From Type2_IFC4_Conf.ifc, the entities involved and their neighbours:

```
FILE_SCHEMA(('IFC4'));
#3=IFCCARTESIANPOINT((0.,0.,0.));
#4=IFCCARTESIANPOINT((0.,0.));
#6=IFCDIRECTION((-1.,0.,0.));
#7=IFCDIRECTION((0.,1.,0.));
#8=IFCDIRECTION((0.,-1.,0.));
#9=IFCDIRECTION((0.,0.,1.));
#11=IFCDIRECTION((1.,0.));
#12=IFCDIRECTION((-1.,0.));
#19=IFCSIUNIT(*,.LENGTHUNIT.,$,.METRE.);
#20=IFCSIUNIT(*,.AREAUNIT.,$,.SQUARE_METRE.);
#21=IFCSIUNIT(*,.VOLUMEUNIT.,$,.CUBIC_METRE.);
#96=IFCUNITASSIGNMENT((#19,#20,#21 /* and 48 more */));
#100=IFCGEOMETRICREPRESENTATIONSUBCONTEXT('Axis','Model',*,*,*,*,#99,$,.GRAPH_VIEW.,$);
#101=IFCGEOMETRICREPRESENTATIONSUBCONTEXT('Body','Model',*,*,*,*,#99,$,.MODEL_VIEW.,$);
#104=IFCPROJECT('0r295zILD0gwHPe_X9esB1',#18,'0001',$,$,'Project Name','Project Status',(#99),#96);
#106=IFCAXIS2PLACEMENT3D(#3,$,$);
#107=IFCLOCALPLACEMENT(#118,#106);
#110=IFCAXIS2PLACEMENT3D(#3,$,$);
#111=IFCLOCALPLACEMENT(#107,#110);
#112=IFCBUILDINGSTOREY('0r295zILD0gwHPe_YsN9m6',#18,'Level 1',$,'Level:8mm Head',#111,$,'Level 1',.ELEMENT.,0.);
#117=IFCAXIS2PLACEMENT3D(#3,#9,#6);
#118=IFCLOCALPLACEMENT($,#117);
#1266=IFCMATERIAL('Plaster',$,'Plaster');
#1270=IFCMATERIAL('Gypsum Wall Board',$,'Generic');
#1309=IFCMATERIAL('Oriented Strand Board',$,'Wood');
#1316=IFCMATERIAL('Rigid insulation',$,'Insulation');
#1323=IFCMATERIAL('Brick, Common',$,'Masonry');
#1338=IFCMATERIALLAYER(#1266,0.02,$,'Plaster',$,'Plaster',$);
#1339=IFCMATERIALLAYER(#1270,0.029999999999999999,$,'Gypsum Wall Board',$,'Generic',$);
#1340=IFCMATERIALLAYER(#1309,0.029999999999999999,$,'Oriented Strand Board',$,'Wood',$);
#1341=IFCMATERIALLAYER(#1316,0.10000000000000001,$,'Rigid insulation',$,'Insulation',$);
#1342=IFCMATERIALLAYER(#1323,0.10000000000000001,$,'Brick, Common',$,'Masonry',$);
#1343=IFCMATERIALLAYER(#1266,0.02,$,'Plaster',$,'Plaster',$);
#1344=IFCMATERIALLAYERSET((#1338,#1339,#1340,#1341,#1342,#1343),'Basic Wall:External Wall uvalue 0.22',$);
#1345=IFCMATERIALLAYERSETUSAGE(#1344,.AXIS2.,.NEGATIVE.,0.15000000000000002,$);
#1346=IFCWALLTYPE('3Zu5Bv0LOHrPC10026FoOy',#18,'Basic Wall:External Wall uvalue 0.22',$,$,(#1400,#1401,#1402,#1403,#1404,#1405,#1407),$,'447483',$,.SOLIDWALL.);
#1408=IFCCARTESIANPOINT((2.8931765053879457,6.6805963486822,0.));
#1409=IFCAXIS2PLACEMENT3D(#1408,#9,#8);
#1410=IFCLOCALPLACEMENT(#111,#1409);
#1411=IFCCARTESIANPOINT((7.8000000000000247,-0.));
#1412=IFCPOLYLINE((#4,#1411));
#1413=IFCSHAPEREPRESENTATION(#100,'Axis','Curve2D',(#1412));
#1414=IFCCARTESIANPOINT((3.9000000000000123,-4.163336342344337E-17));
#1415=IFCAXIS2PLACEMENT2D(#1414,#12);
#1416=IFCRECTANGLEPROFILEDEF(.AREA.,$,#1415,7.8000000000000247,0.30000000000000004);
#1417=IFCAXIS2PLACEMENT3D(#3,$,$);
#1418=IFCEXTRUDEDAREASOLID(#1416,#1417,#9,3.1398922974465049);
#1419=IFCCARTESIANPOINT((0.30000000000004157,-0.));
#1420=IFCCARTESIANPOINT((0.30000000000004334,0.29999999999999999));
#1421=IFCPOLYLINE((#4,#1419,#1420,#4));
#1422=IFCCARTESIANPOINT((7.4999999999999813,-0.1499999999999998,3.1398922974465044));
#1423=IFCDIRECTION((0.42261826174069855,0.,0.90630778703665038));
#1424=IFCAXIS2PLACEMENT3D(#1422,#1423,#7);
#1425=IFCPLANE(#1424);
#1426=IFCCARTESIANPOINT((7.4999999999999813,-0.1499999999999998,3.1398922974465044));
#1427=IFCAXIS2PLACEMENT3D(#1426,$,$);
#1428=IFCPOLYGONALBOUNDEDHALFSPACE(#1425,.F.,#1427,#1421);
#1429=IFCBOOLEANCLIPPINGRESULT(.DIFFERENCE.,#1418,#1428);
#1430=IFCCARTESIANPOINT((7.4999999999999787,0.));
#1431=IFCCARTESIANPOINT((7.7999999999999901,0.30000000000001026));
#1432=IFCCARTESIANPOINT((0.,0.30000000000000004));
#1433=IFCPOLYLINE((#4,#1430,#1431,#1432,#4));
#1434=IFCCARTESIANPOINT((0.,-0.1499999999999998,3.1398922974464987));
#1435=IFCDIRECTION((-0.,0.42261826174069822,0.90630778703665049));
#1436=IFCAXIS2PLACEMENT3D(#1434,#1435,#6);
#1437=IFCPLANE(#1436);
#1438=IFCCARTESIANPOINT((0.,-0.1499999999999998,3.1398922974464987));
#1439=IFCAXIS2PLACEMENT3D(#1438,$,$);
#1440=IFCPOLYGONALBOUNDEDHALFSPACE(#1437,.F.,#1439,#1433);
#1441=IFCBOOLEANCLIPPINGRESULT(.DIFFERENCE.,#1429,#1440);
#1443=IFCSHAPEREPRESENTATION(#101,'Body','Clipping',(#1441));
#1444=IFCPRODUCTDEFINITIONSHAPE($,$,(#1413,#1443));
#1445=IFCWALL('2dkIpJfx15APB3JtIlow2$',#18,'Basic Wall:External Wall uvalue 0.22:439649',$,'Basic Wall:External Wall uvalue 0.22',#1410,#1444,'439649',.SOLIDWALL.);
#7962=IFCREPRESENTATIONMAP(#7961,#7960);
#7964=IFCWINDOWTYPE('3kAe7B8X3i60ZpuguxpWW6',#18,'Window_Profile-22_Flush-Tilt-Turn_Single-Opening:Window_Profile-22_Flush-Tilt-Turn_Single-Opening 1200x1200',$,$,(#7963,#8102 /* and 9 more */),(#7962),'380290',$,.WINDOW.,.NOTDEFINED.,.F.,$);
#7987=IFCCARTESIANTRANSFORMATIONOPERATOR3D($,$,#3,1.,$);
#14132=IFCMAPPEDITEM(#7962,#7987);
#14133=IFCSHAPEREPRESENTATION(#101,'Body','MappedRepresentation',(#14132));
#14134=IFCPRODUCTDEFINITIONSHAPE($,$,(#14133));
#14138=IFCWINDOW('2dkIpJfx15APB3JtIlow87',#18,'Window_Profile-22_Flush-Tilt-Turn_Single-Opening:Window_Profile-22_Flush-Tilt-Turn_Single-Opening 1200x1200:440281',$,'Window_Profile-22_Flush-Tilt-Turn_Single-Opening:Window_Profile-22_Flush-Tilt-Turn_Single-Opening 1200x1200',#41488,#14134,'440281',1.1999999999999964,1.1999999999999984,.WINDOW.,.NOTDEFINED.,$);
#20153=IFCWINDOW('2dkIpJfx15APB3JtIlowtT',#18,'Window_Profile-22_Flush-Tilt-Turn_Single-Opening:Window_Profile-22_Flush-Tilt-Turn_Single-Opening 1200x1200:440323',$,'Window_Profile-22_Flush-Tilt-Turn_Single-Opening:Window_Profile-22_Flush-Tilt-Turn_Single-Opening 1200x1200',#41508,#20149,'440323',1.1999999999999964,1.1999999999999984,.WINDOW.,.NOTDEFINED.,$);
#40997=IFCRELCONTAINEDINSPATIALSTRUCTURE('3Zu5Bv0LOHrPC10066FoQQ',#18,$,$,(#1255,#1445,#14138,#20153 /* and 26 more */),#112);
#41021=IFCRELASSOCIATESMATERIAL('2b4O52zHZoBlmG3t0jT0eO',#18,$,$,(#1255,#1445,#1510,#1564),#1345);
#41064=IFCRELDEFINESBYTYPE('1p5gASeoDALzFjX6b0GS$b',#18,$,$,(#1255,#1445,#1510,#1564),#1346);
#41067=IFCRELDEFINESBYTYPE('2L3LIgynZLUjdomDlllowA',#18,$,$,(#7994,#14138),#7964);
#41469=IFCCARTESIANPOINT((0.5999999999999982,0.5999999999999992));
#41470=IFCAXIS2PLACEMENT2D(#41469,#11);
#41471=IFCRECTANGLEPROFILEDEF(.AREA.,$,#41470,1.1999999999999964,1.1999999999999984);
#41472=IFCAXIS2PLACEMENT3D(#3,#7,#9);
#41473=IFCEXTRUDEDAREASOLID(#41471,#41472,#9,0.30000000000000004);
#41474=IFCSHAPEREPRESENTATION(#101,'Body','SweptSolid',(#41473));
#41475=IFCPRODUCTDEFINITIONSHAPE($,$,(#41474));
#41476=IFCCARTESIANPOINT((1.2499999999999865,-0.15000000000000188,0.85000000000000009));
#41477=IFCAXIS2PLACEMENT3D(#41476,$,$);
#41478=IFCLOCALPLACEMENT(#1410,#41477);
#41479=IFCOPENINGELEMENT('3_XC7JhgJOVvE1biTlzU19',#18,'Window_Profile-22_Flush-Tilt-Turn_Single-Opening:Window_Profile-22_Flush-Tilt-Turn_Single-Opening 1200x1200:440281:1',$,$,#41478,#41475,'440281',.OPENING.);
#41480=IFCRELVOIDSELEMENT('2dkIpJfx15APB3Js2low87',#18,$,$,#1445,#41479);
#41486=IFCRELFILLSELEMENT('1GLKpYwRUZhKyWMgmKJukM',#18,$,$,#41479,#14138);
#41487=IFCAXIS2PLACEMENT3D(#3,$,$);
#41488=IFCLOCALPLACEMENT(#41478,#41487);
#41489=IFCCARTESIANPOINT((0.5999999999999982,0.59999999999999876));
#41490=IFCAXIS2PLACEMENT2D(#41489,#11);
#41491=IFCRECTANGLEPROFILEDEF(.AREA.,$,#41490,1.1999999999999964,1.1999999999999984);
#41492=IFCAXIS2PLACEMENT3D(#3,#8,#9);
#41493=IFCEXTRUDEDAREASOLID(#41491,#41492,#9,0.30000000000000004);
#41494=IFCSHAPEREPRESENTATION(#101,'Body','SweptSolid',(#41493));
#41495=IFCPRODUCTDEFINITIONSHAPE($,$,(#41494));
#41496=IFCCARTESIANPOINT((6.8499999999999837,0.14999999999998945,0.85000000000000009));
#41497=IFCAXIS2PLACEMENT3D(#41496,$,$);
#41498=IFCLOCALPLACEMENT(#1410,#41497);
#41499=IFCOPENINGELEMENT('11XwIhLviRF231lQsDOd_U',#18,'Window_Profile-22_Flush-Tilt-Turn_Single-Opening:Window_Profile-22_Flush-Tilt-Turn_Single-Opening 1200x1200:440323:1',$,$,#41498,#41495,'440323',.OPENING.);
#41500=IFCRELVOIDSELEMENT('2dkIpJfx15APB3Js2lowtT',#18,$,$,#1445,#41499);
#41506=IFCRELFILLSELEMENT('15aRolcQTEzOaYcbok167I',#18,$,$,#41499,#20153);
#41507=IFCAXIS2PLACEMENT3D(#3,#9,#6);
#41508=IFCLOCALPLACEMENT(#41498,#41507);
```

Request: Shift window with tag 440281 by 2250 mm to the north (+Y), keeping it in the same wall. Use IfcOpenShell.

```python
import ifcopenshell
import ifcopenshell.api.geometry
import ifcopenshell.util.placement

model = ifcopenshell.open("Type2_IFC4_Conf.ifc")

window = model.by_id(14138)
opening = window.FillsVoids[0].RelatingOpeningElement
wall = opening.VoidsElements[0].RelatingBuildingElement

wall_matrix = ifcopenshell.util.placement.get_local_placement(wall.ObjectPlacement)
shift = wall_matrix[:3, 0] * 2.25
before = ifcopenshell.util.placement.get_local_placement(window.ObjectPlacement)[:3, 3].copy()

# The window is placed relative to its opening, so it follows when the opening moves.
matrix = ifcopenshell.util.placement.get_local_placement(opening.ObjectPlacement)
matrix[:3, 3] += shift
ifcopenshell.api.geometry.edit_object_placement(
    model, product=opening, matrix=matrix, is_si=False, should_transform_children=True
)

after = ifcopenshell.util.placement.get_local_placement(window.ObjectPlacement)[:3, 3]
print("window moved by", (after - before).round(3) + 0.0)

model.write("Type2_IFC4_Conf-out.ifc")
```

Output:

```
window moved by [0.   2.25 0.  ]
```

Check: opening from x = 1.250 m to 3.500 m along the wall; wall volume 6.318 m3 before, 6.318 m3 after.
